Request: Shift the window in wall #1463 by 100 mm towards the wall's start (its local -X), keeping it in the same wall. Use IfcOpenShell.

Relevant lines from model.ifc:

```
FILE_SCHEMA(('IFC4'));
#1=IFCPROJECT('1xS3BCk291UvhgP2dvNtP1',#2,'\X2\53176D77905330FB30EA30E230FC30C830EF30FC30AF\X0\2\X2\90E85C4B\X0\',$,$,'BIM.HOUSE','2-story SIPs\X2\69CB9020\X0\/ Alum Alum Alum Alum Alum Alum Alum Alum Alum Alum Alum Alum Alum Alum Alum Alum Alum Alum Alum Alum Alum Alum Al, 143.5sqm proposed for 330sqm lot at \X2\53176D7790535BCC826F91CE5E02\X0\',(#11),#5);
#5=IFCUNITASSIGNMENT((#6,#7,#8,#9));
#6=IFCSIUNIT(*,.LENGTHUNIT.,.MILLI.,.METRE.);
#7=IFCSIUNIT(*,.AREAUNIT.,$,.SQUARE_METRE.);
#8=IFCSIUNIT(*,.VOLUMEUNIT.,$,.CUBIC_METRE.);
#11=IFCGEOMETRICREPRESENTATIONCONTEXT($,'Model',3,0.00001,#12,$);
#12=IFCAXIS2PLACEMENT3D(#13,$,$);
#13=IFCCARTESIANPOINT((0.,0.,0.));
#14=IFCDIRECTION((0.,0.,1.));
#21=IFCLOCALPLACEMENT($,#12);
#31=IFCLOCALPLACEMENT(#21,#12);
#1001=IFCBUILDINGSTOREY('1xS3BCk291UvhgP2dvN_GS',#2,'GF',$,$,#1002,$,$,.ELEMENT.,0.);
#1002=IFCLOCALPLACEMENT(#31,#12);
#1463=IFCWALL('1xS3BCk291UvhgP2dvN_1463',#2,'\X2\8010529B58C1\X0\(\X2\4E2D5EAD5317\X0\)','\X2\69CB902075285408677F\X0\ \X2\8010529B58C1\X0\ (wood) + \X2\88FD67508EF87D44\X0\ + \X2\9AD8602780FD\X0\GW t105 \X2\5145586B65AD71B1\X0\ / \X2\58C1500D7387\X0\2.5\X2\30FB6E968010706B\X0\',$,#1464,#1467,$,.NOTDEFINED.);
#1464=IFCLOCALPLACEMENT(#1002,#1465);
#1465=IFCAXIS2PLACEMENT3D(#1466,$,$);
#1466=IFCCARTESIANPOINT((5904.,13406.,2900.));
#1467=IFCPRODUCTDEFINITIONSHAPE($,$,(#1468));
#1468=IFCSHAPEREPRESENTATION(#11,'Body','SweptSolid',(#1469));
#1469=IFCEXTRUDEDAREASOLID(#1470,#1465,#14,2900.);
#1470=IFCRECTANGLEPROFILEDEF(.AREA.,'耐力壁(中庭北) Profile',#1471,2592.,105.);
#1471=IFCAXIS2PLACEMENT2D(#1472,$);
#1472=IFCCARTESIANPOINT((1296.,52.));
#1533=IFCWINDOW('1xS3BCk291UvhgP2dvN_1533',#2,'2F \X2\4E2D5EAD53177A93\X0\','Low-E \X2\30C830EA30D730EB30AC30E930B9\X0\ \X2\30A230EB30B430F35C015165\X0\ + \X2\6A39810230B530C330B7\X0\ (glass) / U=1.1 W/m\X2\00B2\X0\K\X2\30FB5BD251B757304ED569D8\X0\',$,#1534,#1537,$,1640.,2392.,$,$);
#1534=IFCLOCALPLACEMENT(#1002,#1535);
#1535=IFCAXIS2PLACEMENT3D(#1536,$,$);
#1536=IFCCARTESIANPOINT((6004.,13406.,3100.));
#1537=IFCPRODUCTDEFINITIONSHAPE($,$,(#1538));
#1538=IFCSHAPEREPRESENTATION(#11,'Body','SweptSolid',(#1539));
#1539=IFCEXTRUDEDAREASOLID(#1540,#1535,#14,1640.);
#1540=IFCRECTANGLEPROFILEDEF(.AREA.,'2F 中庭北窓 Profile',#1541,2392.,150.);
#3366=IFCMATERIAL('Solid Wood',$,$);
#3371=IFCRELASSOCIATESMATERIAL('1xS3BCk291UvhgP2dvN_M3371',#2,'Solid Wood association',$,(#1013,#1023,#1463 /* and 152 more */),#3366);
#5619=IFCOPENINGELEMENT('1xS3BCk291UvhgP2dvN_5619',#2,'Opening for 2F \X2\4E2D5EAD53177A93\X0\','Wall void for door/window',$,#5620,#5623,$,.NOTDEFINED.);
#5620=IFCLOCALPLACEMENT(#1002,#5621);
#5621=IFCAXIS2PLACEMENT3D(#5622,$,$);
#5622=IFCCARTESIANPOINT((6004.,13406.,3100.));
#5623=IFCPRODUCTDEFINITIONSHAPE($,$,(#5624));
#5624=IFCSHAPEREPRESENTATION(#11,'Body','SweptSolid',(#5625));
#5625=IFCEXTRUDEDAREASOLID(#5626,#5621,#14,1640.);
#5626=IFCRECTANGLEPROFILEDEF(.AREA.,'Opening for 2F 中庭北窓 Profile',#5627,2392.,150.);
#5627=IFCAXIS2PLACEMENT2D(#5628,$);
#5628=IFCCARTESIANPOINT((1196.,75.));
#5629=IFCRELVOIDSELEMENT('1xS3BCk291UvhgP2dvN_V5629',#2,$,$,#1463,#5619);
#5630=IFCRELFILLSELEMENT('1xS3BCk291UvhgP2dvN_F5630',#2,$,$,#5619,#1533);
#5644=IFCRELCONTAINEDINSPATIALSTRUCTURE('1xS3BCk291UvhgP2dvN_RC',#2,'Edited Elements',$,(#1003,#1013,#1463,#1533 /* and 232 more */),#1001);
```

```python
import ifcopenshell
import ifcopenshell.api.geometry
import ifcopenshell.util.placement
import ifcopenshell.util.unit

model = ifcopenshell.open("model.ifc")
unit_scale = ifcopenshell.util.unit.calculate_unit_scale(model)

window = model.by_guid("1xS3BCk291UvhgP2dvN_1533")
opening = window.FillsVoids[0].RelatingOpeningElement
wall = opening.VoidsElements[0].RelatingBuildingElement

wall_matrix = ifcopenshell.util.placement.get_local_placement(wall.ObjectPlacement)
shift = wall_matrix[:3, 0] * -0.1 / unit_scale
before = ifcopenshell.util.placement.get_local_placement(window.ObjectPlacement)[:3, 3].copy()

# The window is not placed relative to its opening, so move both.
for product in (opening, window):
    matrix = ifcopenshell.util.placement.get_local_placement(product.ObjectPlacement)
    matrix[:3, 3] += shift
    ifcopenshell.api.geometry.edit_object_placement(model, product=product, matrix=matrix, is_si=False)

after = ifcopenshell.util.placement.get_local_placement(window.ObjectPlacement)[:3, 3]
print("window moved by", (after - before).round(3) + 0.0)

model.write("model-out.ifc")
```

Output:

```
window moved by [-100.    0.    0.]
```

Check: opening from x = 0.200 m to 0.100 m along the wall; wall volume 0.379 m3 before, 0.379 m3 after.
